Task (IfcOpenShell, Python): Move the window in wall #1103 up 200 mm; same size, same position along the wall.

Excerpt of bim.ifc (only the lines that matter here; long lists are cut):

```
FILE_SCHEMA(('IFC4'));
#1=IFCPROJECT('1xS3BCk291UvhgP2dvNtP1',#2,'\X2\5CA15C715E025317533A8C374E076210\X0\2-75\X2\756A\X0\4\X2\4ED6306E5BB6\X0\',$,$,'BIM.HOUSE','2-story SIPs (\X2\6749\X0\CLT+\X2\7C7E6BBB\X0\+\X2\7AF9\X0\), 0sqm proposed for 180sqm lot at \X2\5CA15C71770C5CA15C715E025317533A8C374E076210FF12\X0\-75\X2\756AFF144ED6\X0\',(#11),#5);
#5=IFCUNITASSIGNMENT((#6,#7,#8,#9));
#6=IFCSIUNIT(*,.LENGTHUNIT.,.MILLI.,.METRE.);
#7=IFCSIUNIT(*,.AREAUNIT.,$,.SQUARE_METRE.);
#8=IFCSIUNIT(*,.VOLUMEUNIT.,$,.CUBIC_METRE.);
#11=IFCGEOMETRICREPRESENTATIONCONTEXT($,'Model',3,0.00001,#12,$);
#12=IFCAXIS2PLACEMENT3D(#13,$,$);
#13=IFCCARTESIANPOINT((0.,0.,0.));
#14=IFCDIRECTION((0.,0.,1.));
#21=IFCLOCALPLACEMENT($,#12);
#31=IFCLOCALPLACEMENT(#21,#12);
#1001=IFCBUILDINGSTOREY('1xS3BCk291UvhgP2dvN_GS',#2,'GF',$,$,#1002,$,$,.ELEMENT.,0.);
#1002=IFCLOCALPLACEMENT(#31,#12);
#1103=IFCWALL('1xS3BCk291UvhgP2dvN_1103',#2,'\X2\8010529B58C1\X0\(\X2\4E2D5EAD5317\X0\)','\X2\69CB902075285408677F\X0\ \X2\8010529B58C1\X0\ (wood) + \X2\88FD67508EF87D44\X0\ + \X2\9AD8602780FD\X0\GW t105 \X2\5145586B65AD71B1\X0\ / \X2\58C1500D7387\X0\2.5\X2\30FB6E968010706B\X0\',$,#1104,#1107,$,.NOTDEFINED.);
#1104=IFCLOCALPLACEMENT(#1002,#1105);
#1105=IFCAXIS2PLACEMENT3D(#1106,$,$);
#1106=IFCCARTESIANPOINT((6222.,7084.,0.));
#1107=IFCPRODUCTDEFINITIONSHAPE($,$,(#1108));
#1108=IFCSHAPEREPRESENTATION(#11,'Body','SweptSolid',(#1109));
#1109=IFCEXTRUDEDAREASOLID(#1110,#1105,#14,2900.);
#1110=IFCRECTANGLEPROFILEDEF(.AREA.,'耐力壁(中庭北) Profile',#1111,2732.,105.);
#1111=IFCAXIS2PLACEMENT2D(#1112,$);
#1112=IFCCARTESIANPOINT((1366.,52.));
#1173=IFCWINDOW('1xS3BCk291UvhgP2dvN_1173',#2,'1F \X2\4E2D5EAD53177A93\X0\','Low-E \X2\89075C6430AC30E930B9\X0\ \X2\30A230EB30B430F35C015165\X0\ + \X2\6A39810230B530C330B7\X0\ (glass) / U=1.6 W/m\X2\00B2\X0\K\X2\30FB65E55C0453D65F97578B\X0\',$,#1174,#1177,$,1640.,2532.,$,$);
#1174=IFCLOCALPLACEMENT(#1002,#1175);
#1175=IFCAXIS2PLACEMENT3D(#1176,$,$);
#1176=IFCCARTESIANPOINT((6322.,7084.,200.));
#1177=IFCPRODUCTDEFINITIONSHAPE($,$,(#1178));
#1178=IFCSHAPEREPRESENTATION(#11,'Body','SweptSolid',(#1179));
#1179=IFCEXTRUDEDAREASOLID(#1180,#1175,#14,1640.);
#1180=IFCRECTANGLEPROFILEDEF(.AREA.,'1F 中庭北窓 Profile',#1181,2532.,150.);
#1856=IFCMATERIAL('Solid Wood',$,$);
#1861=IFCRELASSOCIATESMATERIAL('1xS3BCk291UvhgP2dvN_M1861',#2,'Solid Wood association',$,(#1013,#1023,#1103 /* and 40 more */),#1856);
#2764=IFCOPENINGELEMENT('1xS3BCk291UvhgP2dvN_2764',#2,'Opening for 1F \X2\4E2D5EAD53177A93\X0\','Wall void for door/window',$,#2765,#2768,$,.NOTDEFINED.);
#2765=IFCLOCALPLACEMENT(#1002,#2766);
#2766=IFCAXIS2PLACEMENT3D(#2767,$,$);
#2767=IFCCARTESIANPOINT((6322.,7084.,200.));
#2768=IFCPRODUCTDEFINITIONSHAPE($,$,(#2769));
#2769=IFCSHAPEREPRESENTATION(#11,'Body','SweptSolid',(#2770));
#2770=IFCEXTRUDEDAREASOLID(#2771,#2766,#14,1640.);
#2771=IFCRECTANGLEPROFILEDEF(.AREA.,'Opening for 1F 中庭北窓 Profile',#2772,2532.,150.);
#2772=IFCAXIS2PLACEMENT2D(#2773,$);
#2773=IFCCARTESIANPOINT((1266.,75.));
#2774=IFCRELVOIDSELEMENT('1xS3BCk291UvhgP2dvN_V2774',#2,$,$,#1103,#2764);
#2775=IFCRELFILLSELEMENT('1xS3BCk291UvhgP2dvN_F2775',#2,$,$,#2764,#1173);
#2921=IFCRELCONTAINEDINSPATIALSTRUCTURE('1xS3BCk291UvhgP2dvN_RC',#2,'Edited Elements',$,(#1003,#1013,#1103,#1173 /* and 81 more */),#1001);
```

```python
import numpy as np
import ifcopenshell
import ifcopenshell.api.geometry
import ifcopenshell.util.placement
import ifcopenshell.util.unit

model = ifcopenshell.open("bim.ifc")
unit_scale = ifcopenshell.util.unit.calculate_unit_scale(model)

window = model.by_guid("1xS3BCk291UvhgP2dvN_1173")
opening = window.FillsVoids[0].RelatingOpeningElement
dz = 0.2 / unit_scale

shift = np.array([0.0, 0.0, dz])
# The window is not placed relative to its opening, so move both.
for product in (opening, window):
    matrix = ifcopenshell.util.placement.get_local_placement(product.ObjectPlacement)
    matrix[:3, 3] += shift
    ifcopenshell.api.geometry.edit_object_placement(model, product=product, matrix=matrix, is_si=False)

print(f"moved by {dz * unit_scale:+.3f} m")

model.write("bim_edited.ifc")
```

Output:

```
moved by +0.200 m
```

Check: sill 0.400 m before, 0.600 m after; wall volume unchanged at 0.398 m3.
